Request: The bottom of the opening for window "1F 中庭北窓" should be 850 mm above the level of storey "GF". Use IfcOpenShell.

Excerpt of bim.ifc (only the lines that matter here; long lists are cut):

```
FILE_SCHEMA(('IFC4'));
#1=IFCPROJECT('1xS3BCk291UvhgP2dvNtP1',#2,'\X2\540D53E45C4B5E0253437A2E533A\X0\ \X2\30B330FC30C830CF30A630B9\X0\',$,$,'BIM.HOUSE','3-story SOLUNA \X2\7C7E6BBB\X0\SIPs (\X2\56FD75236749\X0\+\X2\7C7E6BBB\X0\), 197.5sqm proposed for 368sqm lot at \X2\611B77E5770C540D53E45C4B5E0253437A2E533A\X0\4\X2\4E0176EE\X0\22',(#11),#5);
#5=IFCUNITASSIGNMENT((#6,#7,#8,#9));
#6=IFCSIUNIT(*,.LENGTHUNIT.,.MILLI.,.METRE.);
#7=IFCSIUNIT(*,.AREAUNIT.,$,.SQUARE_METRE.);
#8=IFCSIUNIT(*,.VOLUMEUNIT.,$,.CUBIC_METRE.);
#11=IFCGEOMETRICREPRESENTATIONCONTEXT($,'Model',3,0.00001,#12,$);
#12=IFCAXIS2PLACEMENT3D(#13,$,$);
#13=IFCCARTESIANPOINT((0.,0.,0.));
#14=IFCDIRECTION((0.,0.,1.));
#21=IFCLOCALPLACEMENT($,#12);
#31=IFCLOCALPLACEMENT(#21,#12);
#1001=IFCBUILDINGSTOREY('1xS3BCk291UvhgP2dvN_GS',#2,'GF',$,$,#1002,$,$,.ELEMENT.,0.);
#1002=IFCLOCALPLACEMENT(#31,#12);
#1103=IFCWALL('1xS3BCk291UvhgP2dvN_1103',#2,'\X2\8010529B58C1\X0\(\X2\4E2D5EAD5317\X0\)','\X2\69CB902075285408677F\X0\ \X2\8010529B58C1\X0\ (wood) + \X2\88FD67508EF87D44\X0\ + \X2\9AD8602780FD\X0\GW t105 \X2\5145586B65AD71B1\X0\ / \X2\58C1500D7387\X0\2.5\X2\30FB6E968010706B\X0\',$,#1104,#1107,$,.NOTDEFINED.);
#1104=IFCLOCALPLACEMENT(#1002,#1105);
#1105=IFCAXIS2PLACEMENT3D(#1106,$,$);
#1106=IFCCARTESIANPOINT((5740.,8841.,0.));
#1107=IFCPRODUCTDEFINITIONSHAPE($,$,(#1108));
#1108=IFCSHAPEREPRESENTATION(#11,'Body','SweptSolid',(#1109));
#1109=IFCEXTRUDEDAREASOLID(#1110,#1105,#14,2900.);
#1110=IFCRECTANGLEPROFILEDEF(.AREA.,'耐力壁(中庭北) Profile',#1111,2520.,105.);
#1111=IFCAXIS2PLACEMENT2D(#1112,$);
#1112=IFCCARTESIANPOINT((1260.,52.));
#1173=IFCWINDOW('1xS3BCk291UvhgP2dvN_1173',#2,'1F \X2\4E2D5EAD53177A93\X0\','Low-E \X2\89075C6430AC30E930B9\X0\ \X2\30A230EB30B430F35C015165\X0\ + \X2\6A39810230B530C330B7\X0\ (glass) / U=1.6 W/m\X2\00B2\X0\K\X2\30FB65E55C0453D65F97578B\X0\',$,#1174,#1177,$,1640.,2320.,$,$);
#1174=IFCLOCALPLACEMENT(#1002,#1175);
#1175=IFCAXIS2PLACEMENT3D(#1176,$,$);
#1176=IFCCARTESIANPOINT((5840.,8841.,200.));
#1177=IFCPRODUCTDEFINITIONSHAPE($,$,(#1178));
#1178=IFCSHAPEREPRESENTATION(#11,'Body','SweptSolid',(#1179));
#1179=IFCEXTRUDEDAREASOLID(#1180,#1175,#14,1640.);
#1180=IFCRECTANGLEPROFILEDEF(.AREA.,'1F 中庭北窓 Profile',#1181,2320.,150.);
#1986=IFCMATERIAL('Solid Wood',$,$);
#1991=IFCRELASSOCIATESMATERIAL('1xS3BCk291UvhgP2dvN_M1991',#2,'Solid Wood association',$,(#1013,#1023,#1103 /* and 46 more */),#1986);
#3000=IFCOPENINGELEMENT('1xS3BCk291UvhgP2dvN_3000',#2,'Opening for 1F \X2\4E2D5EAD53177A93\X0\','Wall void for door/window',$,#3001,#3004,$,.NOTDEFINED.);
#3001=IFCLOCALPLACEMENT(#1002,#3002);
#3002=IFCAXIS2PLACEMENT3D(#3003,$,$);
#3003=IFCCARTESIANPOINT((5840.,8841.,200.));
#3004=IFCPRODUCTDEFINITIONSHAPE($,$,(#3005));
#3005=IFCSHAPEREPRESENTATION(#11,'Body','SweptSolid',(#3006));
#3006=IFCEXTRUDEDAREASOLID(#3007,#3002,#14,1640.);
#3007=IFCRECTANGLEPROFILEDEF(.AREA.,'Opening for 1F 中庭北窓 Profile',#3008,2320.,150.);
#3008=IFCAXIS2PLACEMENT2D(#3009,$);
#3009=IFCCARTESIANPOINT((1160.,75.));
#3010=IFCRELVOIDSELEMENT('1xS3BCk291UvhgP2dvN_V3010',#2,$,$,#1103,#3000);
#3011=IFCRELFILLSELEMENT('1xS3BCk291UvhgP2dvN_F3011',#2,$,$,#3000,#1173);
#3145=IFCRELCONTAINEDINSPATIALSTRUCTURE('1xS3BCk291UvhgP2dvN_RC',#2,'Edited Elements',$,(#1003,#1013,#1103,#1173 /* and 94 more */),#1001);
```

```python
import numpy as np
import ifcopenshell
import ifcopenshell.api.geometry
import ifcopenshell.geom
import ifcopenshell.util.element
import ifcopenshell.util.placement
import ifcopenshell.util.shape
import ifcopenshell.util.unit

model = ifcopenshell.open("bim.ifc")
unit_scale = ifcopenshell.util.unit.calculate_unit_scale(model)

window = model.by_id(1173)
opening = window.FillsVoids[0].RelatingOpeningElement
storey = ifcopenshell.util.element.get_container(window, ifc_class="IfcBuildingStorey")
level = ifcopenshell.util.placement.get_local_placement(storey.ObjectPlacement)[2, 3]

# The opening's origin need not be at the sill, so measure its lowest point.
shape = ifcopenshell.geom.create_shape(ifcopenshell.geom.settings(), opening)
bottom = ifcopenshell.util.shape.get_shape_bottom_elevation(shape, shape.geometry) / unit_scale
dz = level + 850.0 - bottom

shift = np.array([0.0, 0.0, dz])
# The window is not placed relative to its opening, so move both.
for product in (opening, window):
    matrix = ifcopenshell.util.placement.get_local_placement(product.ObjectPlacement)
    matrix[:3, 3] += shift
    ifcopenshell.api.geometry.edit_object_placement(model, product=product, matrix=matrix, is_si=False)

print(f"moved by {dz * unit_scale:+.3f} m")

model.write("bim_v2.ifc")
```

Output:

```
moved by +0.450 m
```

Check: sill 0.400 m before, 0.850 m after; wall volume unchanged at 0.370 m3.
